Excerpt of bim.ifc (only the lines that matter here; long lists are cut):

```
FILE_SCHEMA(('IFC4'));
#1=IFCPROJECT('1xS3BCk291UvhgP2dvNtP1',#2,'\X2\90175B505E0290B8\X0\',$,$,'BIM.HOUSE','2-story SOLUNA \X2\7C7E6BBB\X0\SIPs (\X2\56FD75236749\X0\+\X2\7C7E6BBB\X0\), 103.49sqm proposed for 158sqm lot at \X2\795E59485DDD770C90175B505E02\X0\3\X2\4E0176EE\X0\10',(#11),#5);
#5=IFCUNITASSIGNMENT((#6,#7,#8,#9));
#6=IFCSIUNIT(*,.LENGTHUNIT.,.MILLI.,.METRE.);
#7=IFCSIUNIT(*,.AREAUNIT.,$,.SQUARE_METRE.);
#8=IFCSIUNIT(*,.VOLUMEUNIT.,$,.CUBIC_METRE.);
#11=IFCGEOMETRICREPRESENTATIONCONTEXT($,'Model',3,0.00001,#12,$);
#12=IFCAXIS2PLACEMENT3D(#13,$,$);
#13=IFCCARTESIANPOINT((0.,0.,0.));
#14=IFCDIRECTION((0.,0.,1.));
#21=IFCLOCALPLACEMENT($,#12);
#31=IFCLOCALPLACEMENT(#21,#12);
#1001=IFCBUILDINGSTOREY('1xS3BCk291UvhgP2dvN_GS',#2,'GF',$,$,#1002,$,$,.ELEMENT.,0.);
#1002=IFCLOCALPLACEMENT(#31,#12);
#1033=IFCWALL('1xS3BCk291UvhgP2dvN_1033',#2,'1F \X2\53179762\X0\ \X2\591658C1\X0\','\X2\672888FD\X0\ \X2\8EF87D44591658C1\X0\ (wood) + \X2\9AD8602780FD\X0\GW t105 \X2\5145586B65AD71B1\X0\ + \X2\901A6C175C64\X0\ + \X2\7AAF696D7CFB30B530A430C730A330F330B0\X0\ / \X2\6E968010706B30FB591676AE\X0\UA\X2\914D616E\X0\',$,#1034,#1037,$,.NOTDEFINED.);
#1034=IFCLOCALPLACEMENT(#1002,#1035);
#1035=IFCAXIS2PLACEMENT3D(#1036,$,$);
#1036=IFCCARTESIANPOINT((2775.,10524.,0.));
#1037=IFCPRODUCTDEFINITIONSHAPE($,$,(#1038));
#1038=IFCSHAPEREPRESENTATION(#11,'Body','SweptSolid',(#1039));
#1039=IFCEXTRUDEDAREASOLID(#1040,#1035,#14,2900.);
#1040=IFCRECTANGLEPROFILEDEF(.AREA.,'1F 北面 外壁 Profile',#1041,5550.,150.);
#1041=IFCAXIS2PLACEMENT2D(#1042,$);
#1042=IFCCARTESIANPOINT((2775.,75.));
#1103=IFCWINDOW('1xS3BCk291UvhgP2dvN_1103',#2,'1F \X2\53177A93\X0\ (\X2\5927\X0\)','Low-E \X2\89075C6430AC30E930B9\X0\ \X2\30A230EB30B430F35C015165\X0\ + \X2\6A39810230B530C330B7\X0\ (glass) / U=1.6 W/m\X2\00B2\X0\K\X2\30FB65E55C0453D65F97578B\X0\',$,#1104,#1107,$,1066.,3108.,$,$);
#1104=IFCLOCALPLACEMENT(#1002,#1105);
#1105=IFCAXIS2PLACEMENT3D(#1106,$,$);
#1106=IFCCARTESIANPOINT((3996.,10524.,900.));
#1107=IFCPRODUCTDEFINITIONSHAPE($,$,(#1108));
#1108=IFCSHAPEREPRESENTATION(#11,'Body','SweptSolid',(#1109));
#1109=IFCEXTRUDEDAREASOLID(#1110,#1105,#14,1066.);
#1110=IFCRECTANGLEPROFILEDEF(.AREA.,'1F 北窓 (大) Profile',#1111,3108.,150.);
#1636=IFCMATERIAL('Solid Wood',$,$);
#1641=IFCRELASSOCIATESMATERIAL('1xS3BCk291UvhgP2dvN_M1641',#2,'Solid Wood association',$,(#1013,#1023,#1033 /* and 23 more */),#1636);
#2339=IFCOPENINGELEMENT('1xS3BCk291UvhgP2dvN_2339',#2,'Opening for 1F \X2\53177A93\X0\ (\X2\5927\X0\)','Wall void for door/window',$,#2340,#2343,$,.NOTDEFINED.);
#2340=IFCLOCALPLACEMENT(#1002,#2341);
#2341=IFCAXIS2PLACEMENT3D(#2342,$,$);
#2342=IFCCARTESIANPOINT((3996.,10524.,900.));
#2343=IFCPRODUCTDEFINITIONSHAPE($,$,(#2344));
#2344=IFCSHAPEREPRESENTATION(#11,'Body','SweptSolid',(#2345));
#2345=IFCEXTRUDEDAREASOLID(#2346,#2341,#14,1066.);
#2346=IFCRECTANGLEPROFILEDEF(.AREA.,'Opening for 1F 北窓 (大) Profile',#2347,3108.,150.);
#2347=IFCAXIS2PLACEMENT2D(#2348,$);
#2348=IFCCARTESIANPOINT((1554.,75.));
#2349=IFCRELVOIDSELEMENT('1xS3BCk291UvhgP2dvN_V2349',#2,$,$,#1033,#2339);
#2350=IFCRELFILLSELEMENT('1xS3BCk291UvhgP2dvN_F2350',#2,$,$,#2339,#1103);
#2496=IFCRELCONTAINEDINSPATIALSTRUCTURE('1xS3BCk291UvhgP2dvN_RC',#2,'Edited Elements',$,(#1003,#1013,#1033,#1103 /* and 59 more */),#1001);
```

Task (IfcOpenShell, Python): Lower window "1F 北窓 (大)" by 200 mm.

```python
import numpy as np
import ifcopenshell
import ifcopenshell.api.geometry
import ifcopenshell.util.placement
import ifcopenshell.util.unit

model = ifcopenshell.open("bim.ifc")
unit_scale = ifcopenshell.util.unit.calculate_unit_scale(model)

window = model.by_guid("1xS3BCk291UvhgP2dvN_1103")
opening = window.FillsVoids[0].RelatingOpeningElement
dz = -0.2 / unit_scale

shift = np.array([0.0, 0.0, dz])
# The window is not placed relative to its opening, so move both.
for product in (opening, window):
    matrix = ifcopenshell.util.placement.get_local_placement(product.ObjectPlacement)
    matrix[:3, 3] += shift
    ifcopenshell.api.geometry.edit_object_placement(model, product=product, matrix=matrix, is_si=False)

print(f"moved by {dz * unit_scale:+.3f} m")

model.write("bim_v2.ifc")
```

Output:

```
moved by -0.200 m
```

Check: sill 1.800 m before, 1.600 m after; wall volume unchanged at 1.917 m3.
